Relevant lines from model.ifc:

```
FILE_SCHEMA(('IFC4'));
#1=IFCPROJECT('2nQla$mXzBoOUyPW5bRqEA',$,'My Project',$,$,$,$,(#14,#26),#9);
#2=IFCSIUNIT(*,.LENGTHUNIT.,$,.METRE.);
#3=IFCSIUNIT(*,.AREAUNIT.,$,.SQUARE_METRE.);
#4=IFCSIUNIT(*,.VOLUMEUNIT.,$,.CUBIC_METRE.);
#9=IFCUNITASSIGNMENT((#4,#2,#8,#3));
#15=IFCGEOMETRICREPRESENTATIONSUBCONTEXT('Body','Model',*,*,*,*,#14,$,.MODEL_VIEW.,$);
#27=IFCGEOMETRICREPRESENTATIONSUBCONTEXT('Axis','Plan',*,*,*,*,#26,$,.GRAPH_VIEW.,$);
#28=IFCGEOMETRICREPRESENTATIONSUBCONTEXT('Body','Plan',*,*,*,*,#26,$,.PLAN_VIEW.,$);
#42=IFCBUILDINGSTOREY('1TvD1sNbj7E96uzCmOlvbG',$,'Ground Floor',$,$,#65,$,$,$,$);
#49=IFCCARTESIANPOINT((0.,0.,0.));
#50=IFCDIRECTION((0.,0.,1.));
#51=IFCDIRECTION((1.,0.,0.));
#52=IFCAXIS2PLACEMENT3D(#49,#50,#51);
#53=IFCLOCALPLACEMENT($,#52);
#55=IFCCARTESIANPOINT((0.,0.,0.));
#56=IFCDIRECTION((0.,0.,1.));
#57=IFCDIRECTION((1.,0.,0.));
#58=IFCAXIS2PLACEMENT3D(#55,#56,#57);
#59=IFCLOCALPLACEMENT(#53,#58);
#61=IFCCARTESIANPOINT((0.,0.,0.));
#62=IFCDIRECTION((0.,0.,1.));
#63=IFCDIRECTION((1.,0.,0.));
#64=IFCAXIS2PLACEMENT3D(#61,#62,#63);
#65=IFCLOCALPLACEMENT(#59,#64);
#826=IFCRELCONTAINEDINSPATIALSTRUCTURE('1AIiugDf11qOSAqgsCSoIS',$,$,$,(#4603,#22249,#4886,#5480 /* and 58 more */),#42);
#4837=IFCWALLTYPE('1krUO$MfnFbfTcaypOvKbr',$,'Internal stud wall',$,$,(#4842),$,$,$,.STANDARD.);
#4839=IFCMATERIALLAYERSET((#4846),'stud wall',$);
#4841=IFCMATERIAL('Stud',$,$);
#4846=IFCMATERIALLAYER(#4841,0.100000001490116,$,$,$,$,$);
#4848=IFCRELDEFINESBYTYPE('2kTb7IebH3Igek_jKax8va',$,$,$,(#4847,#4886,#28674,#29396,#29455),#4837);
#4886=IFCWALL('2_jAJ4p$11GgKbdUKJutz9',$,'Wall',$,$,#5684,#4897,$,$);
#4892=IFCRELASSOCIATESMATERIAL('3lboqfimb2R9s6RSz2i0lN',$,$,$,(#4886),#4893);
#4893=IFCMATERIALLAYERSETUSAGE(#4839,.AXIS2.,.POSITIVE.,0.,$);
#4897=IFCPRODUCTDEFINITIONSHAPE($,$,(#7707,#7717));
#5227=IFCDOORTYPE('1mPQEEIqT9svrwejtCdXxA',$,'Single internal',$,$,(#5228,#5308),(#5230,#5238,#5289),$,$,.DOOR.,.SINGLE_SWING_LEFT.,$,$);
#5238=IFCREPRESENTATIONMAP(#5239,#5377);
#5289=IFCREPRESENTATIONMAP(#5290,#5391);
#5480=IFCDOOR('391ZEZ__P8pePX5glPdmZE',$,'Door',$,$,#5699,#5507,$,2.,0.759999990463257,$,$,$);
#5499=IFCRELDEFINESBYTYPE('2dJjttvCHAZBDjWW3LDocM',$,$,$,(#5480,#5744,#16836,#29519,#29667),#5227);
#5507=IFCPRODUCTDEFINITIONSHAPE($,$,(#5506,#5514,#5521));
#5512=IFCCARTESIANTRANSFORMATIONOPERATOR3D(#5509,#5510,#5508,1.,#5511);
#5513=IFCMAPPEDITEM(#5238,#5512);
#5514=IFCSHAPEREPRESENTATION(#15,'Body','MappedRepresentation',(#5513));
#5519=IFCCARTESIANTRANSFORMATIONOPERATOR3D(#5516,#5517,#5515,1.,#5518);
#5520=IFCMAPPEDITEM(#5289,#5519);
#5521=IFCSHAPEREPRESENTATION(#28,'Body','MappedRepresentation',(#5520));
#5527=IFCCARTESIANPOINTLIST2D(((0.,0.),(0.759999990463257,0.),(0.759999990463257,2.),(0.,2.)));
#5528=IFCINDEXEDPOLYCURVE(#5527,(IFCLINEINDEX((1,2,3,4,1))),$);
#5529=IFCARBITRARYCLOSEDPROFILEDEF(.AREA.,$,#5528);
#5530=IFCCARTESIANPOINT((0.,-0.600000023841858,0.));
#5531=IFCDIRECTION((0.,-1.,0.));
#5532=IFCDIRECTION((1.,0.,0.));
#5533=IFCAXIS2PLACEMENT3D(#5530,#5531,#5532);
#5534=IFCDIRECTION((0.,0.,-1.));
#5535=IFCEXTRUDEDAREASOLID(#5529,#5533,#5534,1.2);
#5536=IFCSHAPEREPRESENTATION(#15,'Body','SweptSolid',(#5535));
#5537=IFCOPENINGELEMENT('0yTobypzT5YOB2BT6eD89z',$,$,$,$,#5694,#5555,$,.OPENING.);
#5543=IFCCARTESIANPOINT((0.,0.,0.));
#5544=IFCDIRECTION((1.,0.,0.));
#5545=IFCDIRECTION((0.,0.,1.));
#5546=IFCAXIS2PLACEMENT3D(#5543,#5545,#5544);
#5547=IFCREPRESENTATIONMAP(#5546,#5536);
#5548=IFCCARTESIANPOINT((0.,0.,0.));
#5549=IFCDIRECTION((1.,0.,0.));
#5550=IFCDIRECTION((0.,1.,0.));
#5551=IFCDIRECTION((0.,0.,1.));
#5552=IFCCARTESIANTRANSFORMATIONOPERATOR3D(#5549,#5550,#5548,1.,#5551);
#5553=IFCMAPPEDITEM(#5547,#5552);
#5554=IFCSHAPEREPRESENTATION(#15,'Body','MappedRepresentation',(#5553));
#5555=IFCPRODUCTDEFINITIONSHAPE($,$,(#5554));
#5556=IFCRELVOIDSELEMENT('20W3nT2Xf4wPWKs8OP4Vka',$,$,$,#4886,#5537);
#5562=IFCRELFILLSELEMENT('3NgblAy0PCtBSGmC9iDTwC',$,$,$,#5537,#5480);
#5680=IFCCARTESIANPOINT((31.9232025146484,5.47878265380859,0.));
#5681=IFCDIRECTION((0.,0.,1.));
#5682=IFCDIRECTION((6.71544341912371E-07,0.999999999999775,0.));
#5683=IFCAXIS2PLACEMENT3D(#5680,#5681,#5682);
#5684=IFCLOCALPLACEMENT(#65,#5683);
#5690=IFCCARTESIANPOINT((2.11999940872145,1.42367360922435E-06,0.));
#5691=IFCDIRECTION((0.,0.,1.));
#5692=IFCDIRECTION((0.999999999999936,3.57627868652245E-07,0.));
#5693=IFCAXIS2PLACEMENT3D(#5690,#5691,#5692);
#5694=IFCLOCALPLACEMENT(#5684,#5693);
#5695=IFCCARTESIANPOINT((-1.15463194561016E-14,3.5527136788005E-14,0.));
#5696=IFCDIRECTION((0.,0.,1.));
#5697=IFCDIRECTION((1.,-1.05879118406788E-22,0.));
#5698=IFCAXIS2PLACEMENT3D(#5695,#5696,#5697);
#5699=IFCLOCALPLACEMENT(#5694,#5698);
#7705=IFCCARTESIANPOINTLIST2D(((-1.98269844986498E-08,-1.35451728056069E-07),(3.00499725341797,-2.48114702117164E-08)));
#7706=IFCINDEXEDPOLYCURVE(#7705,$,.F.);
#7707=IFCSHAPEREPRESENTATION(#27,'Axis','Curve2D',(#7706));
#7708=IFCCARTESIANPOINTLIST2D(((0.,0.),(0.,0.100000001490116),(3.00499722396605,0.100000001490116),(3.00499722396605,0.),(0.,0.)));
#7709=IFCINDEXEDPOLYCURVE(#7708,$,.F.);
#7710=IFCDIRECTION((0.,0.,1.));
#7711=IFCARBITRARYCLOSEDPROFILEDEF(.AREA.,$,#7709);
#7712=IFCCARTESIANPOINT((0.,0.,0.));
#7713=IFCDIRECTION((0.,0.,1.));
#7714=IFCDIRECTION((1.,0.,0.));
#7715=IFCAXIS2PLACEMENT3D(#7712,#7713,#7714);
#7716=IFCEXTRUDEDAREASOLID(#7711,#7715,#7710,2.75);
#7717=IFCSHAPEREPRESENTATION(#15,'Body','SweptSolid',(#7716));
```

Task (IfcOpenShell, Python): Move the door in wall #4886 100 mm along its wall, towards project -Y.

```python
import ifcopenshell
import ifcopenshell.api.geometry
import ifcopenshell.util.placement

model = ifcopenshell.open("model.ifc")

door = model.by_guid("391ZEZ__P8pePX5glPdmZE")
opening = door.FillsVoids[0].RelatingOpeningElement
wall = opening.VoidsElements[0].RelatingBuildingElement

wall_matrix = ifcopenshell.util.placement.get_local_placement(wall.ObjectPlacement)
shift = wall_matrix[:3, 0] * -0.1
before = ifcopenshell.util.placement.get_local_placement(door.ObjectPlacement)[:3, 3].copy()

# The door is placed relative to its opening, so it follows when the opening moves.
matrix = ifcopenshell.util.placement.get_local_placement(opening.ObjectPlacement)
matrix[:3, 3] += shift
ifcopenshell.api.geometry.edit_object_placement(
    model, product=opening, matrix=matrix, is_si=False, should_transform_children=True
)

after = ifcopenshell.util.placement.get_local_placement(door.ObjectPlacement)[:3, 3]
print("door moved by", (after - before).round(3) + 0.0)

model.write("model_updated.ifc")
```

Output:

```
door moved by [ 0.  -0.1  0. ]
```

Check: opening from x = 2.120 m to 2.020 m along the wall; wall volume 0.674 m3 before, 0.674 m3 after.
